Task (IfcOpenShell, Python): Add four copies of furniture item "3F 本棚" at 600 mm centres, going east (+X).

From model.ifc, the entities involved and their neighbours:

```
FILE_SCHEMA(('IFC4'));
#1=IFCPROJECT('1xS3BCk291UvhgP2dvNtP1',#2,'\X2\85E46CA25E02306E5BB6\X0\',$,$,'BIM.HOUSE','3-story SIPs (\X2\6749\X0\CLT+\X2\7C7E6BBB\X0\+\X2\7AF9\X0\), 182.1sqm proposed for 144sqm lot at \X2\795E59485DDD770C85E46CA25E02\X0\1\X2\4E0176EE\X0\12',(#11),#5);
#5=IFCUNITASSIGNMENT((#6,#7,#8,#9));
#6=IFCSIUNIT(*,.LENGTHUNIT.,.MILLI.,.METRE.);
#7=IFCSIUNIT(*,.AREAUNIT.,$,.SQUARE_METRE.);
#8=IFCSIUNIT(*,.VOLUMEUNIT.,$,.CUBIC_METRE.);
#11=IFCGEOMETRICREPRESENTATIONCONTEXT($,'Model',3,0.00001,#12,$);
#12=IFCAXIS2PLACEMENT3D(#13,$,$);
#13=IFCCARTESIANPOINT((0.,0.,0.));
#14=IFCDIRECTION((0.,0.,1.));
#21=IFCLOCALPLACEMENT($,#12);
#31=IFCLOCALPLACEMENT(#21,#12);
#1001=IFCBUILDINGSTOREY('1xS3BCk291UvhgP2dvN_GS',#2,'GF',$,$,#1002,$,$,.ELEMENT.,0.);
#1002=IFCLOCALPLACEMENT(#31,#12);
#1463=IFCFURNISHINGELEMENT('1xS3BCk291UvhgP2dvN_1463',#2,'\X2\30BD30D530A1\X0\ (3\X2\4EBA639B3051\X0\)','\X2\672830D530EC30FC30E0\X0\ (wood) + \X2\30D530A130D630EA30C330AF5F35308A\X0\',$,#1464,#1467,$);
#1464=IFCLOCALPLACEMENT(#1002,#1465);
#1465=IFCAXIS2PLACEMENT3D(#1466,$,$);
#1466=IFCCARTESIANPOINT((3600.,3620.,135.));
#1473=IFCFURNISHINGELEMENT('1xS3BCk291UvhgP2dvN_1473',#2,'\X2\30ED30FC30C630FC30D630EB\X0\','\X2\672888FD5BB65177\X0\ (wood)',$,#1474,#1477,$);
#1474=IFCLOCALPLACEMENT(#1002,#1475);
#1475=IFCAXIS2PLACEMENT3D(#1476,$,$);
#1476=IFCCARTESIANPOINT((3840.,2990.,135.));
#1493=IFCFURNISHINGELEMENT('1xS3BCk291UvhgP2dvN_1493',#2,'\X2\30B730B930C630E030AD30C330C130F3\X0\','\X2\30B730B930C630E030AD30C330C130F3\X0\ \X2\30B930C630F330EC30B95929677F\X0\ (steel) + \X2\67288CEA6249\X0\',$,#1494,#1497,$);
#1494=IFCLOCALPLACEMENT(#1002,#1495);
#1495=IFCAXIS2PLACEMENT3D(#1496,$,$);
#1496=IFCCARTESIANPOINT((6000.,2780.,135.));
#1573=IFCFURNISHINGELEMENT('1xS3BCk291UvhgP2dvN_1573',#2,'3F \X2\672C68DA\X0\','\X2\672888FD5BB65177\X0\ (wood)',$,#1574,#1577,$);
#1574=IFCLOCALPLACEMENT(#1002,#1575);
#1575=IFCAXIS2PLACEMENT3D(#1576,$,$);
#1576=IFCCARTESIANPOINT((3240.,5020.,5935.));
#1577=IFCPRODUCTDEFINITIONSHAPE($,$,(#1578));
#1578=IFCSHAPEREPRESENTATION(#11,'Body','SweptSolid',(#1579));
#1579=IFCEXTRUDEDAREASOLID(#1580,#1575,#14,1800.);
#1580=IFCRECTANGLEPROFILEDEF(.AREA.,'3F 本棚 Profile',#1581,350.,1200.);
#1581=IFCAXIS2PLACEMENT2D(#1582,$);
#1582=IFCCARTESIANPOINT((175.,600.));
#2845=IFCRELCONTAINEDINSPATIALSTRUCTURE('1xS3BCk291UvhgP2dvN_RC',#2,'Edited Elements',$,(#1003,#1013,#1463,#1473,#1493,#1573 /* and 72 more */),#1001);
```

```python
import numpy as np
import ifcopenshell
import ifcopenshell.api.geometry
import ifcopenshell.api.root
import ifcopenshell.util.element
import ifcopenshell.util.placement

model = ifcopenshell.open("model.ifc")


def reuse_history(source, copy):
    """copy_class also copies each property set's owner history, people and application; keep the originals."""
    for rel in copy.IsDefinedBy:
        if rel.is_a("IfcRelDefinesByProperties") and (history := rel.RelatingPropertyDefinition.OwnerHistory):
            rel.RelatingPropertyDefinition.OwnerHistory = source.OwnerHistory
            ifcopenshell.util.element.remove_deep2(model, history)


source = model.by_id(1573)
base = ifcopenshell.util.placement.get_local_placement(source.ObjectPlacement)
step = np.array([1.0, 0.0, 0.0]) * 600.0

for i in range(1, 5):
    copy = ifcopenshell.api.root.copy_class(model, product=source)
    copy.Representation = ifcopenshell.util.element.copy_deep(
        model, source.Representation, exclude=["IfcGeometricRepresentationContext", "IfcRepresentationMap"]
    )
    reuse_history(source, copy)
    matrix = base.copy()
    matrix[:3, 3] += i * step
    print("added at", matrix[:3, 3].round(3) + 0.0)
    ifcopenshell.api.geometry.edit_object_placement(model, product=copy, matrix=matrix, is_si=False)

model.write("model_v2.ifc")
```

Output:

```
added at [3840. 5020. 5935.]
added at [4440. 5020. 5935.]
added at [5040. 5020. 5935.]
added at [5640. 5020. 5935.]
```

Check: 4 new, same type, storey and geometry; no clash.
